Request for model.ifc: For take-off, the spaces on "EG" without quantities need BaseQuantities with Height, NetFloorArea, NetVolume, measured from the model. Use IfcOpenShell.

First a look at what the model holds.

```python
import ifcopenshell
import ifcopenshell.util.element
import ifcopenshell.util.unit

model = ifcopenshell.open("model.ifc")
print(model.schema)
for unit_type in ("LENGTHUNIT", "AREAUNIT", "VOLUMEUNIT"):
    print(unit_type, ifcopenshell.util.unit.calculate_unit_scale(model, unit_type))
storey = next(s for s in model.by_type("IfcBuildingStorey") if s.Name == "EG")
spaces = [e for e in ifcopenshell.util.element.get_decomposition(storey) if e.is_a("IfcSpace")]
for e in sorted(spaces, key=lambda e: e.id()):
    print(e.id(), e.is_a(), e.Name, list(ifcopenshell.util.element.get_psets(e, qtos_only=True)), sep=" | ")
```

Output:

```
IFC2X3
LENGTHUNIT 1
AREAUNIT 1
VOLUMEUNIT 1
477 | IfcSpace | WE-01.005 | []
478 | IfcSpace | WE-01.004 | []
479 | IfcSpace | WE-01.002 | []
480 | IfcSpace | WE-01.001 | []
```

```python
import ifcopenshell
import ifcopenshell.api.pset
import ifcopenshell.geom
import ifcopenshell.util.element
import ifcopenshell.util.shape
import ifcopenshell.util.unit

model = ifcopenshell.open("model.ifc")
unit_scale = ifcopenshell.util.unit.calculate_unit_scale(model)
area_scale = ifcopenshell.util.unit.calculate_unit_scale(model, "AREAUNIT")
volume_scale = ifcopenshell.util.unit.calculate_unit_scale(model, "VOLUMEUNIT")
settings = ifcopenshell.geom.settings()

storey = next(s for s in model.by_type("IfcBuildingStorey") if s.Name == "EG")
spaces = [e for e in ifcopenshell.util.element.get_decomposition(storey) if e.is_a("IfcSpace")]

for e in sorted(spaces, key=lambda e: e.id()):
    if ifcopenshell.util.element.get_psets(e, qtos_only=True, should_inherit=False):
        continue
    # Geometry comes back in metres, in the element's own axes.
    shape = ifcopenshell.geom.create_shape(settings, e)
    values = {
        "Height": ifcopenshell.util.shape.get_z(shape.geometry) / unit_scale,
        "NetFloorArea": ifcopenshell.util.shape.get_footprint_area(shape.geometry) / area_scale,
        "NetVolume": ifcopenshell.util.shape.get_volume(shape.geometry) / volume_scale,
    }
    qto = ifcopenshell.api.pset.add_qto(model, product=e, name="BaseQuantities")
    ifcopenshell.api.pset.edit_qto(model, qto=qto, properties=values)
    print(e.id(), {k: round(v, 3) for k, v in values.items()})

model.write("model-out.ifc")
```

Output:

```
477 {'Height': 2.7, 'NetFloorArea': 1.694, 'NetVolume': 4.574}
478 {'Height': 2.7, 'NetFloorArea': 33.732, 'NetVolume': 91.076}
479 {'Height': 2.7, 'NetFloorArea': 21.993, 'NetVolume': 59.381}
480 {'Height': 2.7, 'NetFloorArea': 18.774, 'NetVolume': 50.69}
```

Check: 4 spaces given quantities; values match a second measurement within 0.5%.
